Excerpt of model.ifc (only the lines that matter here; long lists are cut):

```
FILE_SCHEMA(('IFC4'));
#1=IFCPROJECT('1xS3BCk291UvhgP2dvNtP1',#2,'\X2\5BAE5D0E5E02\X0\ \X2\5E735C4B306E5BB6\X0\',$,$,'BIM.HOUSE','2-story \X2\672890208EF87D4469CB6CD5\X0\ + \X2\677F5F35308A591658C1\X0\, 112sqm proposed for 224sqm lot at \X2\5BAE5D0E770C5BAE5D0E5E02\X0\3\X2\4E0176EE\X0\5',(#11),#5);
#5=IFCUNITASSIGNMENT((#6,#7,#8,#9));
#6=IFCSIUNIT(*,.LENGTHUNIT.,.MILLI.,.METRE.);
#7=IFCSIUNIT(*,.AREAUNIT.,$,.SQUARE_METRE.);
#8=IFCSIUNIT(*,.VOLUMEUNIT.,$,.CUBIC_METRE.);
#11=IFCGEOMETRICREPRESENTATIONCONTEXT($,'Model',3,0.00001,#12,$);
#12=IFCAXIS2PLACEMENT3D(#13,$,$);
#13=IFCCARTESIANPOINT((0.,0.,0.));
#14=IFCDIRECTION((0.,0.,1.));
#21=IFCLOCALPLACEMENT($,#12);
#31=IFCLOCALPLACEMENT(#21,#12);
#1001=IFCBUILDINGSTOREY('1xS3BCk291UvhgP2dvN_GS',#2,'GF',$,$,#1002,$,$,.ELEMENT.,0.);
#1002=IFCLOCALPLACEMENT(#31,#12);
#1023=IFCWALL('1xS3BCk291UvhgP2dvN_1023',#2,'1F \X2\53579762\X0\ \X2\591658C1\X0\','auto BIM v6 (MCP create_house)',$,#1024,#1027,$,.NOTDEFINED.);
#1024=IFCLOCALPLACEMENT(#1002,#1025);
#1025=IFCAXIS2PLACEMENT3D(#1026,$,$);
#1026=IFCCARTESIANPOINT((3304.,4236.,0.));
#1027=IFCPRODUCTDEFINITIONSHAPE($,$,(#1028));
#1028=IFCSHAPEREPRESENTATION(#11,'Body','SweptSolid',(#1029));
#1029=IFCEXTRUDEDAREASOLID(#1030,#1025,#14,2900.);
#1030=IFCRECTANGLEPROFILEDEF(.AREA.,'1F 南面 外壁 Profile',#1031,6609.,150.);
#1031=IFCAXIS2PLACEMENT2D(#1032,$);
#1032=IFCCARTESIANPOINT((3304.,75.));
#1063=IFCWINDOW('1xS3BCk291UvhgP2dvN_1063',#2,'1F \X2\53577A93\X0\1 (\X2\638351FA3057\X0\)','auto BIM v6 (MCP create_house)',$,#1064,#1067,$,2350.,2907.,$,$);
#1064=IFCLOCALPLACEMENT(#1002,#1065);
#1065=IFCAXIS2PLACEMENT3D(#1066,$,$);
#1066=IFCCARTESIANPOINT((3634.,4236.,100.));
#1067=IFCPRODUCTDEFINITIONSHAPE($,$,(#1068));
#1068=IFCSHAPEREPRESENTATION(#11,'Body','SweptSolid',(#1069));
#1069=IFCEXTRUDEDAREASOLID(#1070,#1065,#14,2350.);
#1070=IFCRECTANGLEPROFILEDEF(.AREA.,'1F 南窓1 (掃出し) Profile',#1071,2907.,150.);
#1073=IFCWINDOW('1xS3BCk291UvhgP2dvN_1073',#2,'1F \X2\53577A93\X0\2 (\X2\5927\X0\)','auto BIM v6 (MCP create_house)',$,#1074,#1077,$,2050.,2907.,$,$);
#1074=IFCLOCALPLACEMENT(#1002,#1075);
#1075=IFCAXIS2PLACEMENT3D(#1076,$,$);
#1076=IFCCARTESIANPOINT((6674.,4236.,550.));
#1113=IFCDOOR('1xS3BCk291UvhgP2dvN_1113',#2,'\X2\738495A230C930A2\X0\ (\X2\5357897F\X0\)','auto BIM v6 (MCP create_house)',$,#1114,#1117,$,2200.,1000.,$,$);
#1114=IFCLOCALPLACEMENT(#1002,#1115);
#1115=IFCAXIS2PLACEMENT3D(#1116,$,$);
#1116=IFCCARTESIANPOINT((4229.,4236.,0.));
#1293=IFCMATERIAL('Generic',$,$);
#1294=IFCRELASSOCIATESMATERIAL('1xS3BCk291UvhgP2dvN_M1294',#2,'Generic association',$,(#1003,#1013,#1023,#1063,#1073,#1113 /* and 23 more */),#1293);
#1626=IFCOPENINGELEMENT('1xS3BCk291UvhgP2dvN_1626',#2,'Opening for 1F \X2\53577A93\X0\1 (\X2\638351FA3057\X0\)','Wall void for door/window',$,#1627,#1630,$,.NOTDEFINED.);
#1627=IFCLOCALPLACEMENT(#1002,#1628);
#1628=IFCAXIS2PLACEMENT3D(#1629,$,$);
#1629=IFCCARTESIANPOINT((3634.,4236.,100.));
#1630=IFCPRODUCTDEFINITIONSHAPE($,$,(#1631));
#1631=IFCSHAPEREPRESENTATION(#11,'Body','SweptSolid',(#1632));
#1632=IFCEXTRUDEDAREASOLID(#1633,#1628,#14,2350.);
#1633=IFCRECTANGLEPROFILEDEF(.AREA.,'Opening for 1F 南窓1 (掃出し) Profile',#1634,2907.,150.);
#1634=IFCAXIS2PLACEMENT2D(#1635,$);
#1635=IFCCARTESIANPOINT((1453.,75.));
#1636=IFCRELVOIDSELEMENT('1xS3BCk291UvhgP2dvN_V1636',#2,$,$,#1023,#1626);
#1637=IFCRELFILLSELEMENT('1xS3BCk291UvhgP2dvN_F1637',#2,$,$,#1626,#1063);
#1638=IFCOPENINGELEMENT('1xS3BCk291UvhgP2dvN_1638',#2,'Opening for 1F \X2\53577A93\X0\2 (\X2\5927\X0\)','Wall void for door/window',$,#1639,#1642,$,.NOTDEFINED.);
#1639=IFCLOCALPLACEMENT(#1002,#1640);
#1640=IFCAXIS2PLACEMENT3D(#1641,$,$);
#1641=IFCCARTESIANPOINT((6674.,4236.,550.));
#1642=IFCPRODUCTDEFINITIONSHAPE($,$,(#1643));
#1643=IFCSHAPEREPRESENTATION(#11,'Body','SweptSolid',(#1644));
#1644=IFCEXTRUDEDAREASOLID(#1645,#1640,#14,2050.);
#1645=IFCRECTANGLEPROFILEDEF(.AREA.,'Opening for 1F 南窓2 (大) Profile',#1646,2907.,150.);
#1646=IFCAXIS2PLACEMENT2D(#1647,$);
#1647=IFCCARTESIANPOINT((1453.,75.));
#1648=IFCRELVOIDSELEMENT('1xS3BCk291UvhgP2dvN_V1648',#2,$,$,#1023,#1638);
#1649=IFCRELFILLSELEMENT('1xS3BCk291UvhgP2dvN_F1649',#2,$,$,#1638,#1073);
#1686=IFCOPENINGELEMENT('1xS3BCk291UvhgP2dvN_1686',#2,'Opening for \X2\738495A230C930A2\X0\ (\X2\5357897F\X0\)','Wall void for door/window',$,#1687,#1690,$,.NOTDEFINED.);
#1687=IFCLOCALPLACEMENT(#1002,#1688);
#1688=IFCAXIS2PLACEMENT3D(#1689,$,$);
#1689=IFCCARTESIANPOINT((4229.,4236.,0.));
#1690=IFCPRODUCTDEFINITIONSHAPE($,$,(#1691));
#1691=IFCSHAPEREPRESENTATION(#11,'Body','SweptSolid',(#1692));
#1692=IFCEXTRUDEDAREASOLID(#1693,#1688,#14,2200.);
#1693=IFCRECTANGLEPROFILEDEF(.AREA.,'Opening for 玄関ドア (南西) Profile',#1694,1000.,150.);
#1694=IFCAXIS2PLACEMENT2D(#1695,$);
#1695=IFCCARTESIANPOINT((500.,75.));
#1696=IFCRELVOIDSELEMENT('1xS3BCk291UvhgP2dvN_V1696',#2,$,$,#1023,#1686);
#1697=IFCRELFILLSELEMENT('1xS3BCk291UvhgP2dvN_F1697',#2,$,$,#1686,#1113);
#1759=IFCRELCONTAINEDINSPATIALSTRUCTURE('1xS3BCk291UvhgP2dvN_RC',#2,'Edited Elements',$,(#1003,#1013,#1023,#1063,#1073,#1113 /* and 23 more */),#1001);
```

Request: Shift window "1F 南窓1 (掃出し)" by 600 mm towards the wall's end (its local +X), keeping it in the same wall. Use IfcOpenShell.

```python
import ifcopenshell
import ifcopenshell.api.geometry
import ifcopenshell.util.placement
import ifcopenshell.util.unit

model = ifcopenshell.open("model.ifc")
unit_scale = ifcopenshell.util.unit.calculate_unit_scale(model)

window = model.by_guid("1xS3BCk291UvhgP2dvN_1063")
opening = window.FillsVoids[0].RelatingOpeningElement
wall = opening.VoidsElements[0].RelatingBuildingElement

wall_matrix = ifcopenshell.util.placement.get_local_placement(wall.ObjectPlacement)
shift = wall_matrix[:3, 0] * 0.6 / unit_scale
before = ifcopenshell.util.placement.get_local_placement(window.ObjectPlacement)[:3, 3].copy()

# The window is not placed relative to its opening, so move both.
for product in (opening, window):
    matrix = ifcopenshell.util.placement.get_local_placement(product.ObjectPlacement)
    matrix[:3, 3] += shift
    ifcopenshell.api.geometry.edit_object_placement(model, product=product, matrix=matrix, is_si=False)

after = ifcopenshell.util.placement.get_local_placement(window.ObjectPlacement)[:3, 3]
print("window moved by", (after - before).round(3) + 0.0)

model.write("model_updated.ifc")
```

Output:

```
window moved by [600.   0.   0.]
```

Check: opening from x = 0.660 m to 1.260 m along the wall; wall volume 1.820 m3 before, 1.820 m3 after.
